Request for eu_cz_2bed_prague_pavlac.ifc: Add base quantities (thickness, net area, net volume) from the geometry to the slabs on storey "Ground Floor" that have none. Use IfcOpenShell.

First a look at what the model holds.

```python
import ifcopenshell
import ifcopenshell.util.element
import ifcopenshell.util.unit

model = ifcopenshell.open("eu_cz_2bed_prague_pavlac.ifc")
print(model.schema)
for unit_type in ("LENGTHUNIT", "AREAUNIT", "VOLUMEUNIT"):
    print(unit_type, ifcopenshell.util.unit.calculate_unit_scale(model, unit_type))
storey = next(s for s in model.by_type("IfcBuildingStorey") if s.Name == "Ground Floor")
slabs = [e for e in ifcopenshell.util.element.get_decomposition(storey) if e.is_a("IfcSlab")]
for e in sorted(slabs, key=lambda e: e.id()):
    print(e.id(), e.is_a(), e.Name, list(ifcopenshell.util.element.get_psets(e, qtos_only=True)), sep=" | ")
```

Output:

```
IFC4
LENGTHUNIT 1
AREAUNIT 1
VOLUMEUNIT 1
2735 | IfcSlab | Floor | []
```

```python
import ifcopenshell
import ifcopenshell.api.pset
import ifcopenshell.geom
import ifcopenshell.util.element
import ifcopenshell.util.shape
import ifcopenshell.util.unit

model = ifcopenshell.open("eu_cz_2bed_prague_pavlac.ifc")
unit_scale = ifcopenshell.util.unit.calculate_unit_scale(model)
area_scale = ifcopenshell.util.unit.calculate_unit_scale(model, "AREAUNIT")
volume_scale = ifcopenshell.util.unit.calculate_unit_scale(model, "VOLUMEUNIT")
settings = ifcopenshell.geom.settings()

storey = next(s for s in model.by_type("IfcBuildingStorey") if s.Name == "Ground Floor")
slabs = [e for e in ifcopenshell.util.element.get_decomposition(storey) if e.is_a("IfcSlab")]

for e in sorted(slabs, key=lambda e: e.id()):
    if ifcopenshell.util.element.get_psets(e, qtos_only=True, should_inherit=False):
        continue
    # Geometry comes back in metres, in the element's own axes.
    shape = ifcopenshell.geom.create_shape(settings, e)
    values = {
        "Width": ifcopenshell.util.shape.get_z(shape.geometry) / unit_scale,
        "NetArea": ifcopenshell.util.shape.get_footprint_area(shape.geometry) / area_scale,
        "NetVolume": ifcopenshell.util.shape.get_volume(shape.geometry) / volume_scale,
    }
    qto = ifcopenshell.api.pset.add_qto(model, product=e, name="Qto_SlabBaseQuantities")
    ifcopenshell.api.pset.edit_qto(model, qto=qto, properties=values)
    print(e.id(), {k: round(v, 3) for k, v in values.items()})

model.write("eu_cz_2bed_prague_pavlac_v2.ifc")
```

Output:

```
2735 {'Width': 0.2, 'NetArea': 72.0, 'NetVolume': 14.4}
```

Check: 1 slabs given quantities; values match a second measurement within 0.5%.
